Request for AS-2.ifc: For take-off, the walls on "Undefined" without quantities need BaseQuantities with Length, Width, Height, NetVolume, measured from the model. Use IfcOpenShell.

First a look at what the model holds.

```python
import ifcopenshell
import ifcopenshell.util.element
import ifcopenshell.util.unit

model = ifcopenshell.open("AS-2.ifc")
print(model.schema)
for unit_type in ("LENGTHUNIT", "AREAUNIT", "VOLUMEUNIT"):
    print(unit_type, ifcopenshell.util.unit.calculate_unit_scale(model, unit_type))
storey = next(s for s in model.by_type("IfcBuildingStorey") if s.Name == "Undefined")
walls = [e for e in ifcopenshell.util.element.get_decomposition(storey) if e.is_a("IfcWall")]
for e in sorted(walls, key=lambda e: e.id()):
    print(e.id(), e.is_a(), e.Name, list(ifcopenshell.util.element.get_psets(e, qtos_only=True)), sep=" | ")
```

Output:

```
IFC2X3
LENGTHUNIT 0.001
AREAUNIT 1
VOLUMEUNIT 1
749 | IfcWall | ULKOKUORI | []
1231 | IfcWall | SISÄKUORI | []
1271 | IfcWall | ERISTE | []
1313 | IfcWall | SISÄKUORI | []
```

```python
import ifcopenshell
import ifcopenshell.api.pset
import ifcopenshell.geom
import ifcopenshell.util.element
import ifcopenshell.util.shape
import ifcopenshell.util.unit

model = ifcopenshell.open("AS-2.ifc")
unit_scale = ifcopenshell.util.unit.calculate_unit_scale(model)
volume_scale = ifcopenshell.util.unit.calculate_unit_scale(model, "VOLUMEUNIT")
settings = ifcopenshell.geom.settings()

storey = next(s for s in model.by_type("IfcBuildingStorey") if s.Name == "Undefined")
walls = [e for e in ifcopenshell.util.element.get_decomposition(storey) if e.is_a("IfcWall")]

for e in sorted(walls, key=lambda e: e.id()):
    if ifcopenshell.util.element.get_psets(e, qtos_only=True, should_inherit=False):
        continue
    # Geometry comes back in metres, in the element's own axes.
    shape = ifcopenshell.geom.create_shape(settings, e)
    values = {
        "Length": ifcopenshell.util.shape.get_x(shape.geometry) / unit_scale,
        "Width": ifcopenshell.util.shape.get_y(shape.geometry) / unit_scale,
        "Height": ifcopenshell.util.shape.get_z(shape.geometry) / unit_scale,
        "NetVolume": ifcopenshell.util.shape.get_volume(shape.geometry) / volume_scale,
    }
    qto = ifcopenshell.api.pset.add_qto(model, product=e, name="BaseQuantities")
    ifcopenshell.api.pset.edit_qto(model, qto=qto, properties=values)
    print(e.id(), {k: round(v, 3) for k, v in values.items()})

model.write("AS-2-out.ifc")
```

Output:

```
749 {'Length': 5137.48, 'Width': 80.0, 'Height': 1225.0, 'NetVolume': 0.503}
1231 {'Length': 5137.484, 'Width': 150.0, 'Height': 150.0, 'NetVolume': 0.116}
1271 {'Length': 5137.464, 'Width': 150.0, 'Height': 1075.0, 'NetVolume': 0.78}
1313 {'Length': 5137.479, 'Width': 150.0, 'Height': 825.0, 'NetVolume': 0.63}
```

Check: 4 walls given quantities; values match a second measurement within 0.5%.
